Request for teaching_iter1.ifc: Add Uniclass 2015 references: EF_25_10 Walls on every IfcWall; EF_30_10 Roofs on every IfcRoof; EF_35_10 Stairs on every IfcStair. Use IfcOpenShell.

First a look at what the model holds.

```python
import ifcopenshell

model = ifcopenshell.open("teaching_iter1.ifc")
print(model.schema)
print("classifications:", [c.Name for c in model.by_type("IfcClassification")])
for ifc_class in ("IfcDoor", "IfcRoof", "IfcStair", "IfcWall", "IfcWindow"):
    print(ifc_class, len(model.by_type(ifc_class)))
```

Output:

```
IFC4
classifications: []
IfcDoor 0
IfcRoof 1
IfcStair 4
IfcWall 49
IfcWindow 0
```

```python
import ifcopenshell
import ifcopenshell.api.classification

model = ifcopenshell.open("teaching_iter1.ifc")

system = ifcopenshell.api.classification.add_classification(model, classification="Uniclass 2015")

codes = {
    "IfcWall": ("EF_25_10", "Walls"),
    "IfcRoof": ("EF_30_10", "Roofs"),
    "IfcStair": ("EF_35_10", "Stairs"),
}
for ifc_class, (code, name) in codes.items():
    products = model.by_type(ifc_class)
    ifcopenshell.api.classification.add_reference(
        model, products=products, classification=system, identification=code, name=name
    )
    print(code, len(products))

model.write("teaching_iter1_rev.ifc")
```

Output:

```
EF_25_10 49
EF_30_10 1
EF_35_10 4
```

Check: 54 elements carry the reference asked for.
